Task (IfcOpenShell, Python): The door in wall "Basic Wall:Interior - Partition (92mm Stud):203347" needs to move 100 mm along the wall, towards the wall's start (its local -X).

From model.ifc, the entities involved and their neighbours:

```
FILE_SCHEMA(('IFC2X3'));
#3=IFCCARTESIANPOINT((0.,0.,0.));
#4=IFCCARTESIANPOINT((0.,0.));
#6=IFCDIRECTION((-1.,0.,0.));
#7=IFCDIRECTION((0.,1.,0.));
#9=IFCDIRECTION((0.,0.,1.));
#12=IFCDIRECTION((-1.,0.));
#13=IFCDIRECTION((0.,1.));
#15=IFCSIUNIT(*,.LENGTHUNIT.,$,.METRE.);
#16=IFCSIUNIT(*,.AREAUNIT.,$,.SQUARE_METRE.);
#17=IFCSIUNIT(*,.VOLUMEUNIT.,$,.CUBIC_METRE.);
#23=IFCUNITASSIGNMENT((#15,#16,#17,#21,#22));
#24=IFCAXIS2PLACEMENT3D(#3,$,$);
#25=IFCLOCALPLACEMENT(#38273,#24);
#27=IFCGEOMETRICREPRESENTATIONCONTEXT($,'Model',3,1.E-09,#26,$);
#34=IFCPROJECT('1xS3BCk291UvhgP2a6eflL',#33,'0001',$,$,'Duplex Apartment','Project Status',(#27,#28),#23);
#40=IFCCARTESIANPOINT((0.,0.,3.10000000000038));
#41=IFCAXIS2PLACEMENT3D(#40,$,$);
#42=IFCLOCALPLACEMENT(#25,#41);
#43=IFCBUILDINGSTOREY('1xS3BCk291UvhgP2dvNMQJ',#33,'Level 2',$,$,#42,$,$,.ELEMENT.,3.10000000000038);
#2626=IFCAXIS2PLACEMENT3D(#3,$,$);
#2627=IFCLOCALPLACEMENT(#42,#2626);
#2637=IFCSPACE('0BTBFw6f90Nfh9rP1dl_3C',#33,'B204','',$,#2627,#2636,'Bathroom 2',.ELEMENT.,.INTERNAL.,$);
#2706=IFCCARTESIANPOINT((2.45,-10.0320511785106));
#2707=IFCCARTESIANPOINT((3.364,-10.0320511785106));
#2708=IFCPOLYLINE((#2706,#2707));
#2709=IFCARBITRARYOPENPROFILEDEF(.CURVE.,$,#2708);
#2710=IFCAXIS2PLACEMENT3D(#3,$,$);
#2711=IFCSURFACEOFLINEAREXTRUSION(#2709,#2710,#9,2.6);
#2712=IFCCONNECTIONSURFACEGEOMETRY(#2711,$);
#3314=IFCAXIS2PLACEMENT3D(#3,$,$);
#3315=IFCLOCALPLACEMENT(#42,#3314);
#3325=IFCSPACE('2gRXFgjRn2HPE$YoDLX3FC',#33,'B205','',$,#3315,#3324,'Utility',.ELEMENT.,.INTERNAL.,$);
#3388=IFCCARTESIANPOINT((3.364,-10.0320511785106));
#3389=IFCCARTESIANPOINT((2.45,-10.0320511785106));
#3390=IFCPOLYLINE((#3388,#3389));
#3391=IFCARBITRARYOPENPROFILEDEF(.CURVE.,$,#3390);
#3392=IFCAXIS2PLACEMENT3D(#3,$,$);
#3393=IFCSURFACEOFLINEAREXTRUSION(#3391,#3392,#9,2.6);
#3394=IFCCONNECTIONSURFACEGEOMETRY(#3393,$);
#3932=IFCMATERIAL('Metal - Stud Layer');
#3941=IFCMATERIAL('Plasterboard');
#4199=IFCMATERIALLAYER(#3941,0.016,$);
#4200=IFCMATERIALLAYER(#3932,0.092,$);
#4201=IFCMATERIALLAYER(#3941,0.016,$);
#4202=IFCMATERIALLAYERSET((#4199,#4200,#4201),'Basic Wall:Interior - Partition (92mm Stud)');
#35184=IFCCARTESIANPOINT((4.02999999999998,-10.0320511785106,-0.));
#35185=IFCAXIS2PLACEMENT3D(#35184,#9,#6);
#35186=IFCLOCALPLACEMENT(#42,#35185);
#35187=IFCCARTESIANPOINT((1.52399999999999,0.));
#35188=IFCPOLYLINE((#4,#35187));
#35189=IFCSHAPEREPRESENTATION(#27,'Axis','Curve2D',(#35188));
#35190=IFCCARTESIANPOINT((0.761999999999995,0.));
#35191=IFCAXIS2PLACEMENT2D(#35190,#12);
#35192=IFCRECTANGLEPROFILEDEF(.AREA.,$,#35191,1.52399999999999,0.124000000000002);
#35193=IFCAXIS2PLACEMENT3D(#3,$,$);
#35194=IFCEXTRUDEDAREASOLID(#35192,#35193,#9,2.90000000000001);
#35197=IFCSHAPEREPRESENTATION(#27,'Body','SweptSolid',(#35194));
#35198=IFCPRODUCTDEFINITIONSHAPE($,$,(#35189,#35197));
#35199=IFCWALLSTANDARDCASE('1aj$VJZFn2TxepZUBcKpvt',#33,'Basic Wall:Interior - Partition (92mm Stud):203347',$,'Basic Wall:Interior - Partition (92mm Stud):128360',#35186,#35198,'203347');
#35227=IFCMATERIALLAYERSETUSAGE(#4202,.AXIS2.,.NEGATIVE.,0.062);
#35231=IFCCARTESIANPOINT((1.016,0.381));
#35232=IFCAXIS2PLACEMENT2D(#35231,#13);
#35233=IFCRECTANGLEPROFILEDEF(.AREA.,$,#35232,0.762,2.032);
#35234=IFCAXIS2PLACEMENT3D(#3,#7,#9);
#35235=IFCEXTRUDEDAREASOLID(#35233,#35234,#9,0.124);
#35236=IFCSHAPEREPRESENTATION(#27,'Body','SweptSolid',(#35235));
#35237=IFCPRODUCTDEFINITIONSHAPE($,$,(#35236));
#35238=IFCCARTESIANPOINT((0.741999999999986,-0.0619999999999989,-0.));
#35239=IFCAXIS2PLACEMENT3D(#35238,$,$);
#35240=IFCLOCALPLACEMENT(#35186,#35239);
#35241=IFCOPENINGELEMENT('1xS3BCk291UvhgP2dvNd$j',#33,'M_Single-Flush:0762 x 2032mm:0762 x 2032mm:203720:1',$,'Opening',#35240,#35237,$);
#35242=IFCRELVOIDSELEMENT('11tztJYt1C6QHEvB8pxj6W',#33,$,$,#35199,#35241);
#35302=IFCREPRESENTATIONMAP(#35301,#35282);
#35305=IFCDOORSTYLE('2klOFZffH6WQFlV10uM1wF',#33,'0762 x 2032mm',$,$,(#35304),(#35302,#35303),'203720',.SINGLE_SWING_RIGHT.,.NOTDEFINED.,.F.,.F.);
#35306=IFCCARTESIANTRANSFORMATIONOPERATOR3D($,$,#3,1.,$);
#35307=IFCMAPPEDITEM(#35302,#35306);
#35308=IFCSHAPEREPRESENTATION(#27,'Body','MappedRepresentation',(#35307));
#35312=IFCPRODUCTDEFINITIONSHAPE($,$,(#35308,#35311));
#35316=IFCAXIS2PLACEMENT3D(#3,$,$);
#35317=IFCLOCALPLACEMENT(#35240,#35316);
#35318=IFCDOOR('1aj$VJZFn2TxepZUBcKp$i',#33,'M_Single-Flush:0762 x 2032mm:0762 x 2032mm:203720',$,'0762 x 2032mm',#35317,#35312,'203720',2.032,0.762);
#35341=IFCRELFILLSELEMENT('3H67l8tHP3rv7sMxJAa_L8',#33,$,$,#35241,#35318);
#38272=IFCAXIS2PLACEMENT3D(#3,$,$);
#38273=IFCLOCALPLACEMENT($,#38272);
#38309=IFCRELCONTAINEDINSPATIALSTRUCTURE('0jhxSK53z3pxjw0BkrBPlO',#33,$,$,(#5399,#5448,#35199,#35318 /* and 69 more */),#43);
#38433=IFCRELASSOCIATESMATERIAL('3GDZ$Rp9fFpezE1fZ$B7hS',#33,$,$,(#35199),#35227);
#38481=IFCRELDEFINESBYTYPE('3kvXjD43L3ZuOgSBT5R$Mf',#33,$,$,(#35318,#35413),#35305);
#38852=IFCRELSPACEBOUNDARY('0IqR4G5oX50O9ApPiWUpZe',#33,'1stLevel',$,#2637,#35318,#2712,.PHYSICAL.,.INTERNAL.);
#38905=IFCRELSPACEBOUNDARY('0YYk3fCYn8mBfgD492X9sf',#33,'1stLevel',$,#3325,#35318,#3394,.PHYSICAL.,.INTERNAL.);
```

```python
import numpy as np
import ifcopenshell
import ifcopenshell.api.geometry
import ifcopenshell.util.placement

model = ifcopenshell.open("model.ifc")

door = model.by_guid("1aj$VJZFn2TxepZUBcKp$i")
opening = door.FillsVoids[0].RelatingOpeningElement
wall = opening.VoidsElements[0].RelatingBuildingElement

wall_matrix = ifcopenshell.util.placement.get_local_placement(wall.ObjectPlacement)
shift = wall_matrix[:3, 0] * -0.1
before = ifcopenshell.util.placement.get_local_placement(door.ObjectPlacement)[:3, 3].copy()

# The door is placed relative to its opening, so it follows when the opening moves.
matrix = ifcopenshell.util.placement.get_local_placement(opening.ObjectPlacement)
matrix[:3, 3] += shift
ifcopenshell.api.geometry.edit_object_placement(
    model, product=opening, matrix=matrix, is_si=False, should_transform_children=True
)

# Space boundary surfaces are stored in each space's coordinates; move them too.
for rel in door.ProvidesBoundaries:
    if not rel.ConnectionGeometry:
        continue
    surface = rel.ConnectionGeometry.SurfaceOnRelatingElement
    space_matrix = ifcopenshell.util.placement.get_local_placement(rel.RelatingSpace.ObjectPlacement)
    point = np.array(surface.Position.Location.Coordinates) + space_matrix[:3, :3].T @ shift
    surface.Position = model.createIfcAxis2Placement3D(
        model.createIfcCartesianPoint(point.tolist()), surface.Position.Axis, surface.Position.RefDirection
    )

after = ifcopenshell.util.placement.get_local_placement(door.ObjectPlacement)[:3, 3]
print("door moved by", (after - before).round(3) + 0.0)

model.write("model_v2.ifc")
```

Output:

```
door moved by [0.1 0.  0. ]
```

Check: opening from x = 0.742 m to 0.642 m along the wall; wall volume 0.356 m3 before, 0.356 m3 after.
